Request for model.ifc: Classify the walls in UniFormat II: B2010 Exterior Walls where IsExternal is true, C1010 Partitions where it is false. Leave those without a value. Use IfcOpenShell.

First a look at what the model holds.

```python
import ifcopenshell
import ifcopenshell.util.element

model = ifcopenshell.open("model.ifc")
print(model.schema)
print("classifications:", [c.Name for c in model.by_type("IfcClassification")])
values = [ifcopenshell.util.element.get_pset(e, "Pset_WallCommon", "IsExternal") for e in model.by_type("IfcWall")]
for value in (True, False, None):
    print("IsExternal", value, values.count(value))
```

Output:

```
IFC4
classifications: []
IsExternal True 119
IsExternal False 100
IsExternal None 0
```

```python
import ifcopenshell
import ifcopenshell.api.classification
import ifcopenshell.util.element

model = ifcopenshell.open("model.ifc")

system = ifcopenshell.api.classification.add_classification(model, classification="UniFormat II")

walls = model.by_type("IfcWall")
external = {e: ifcopenshell.util.element.get_pset(e, "Pset_WallCommon", "IsExternal") for e in walls}
for flag, code, name in ((True, "B2010", "Exterior Walls"), (False, "C1010", "Partitions")):
    products = [e for e in walls if external[e] is flag]
    ifcopenshell.api.classification.add_reference(
        model, products=products, classification=system, identification=code, name=name
    )
    print(code, len(products))

model.write("model_updated.ifc")
```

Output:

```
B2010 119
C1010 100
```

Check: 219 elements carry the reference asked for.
